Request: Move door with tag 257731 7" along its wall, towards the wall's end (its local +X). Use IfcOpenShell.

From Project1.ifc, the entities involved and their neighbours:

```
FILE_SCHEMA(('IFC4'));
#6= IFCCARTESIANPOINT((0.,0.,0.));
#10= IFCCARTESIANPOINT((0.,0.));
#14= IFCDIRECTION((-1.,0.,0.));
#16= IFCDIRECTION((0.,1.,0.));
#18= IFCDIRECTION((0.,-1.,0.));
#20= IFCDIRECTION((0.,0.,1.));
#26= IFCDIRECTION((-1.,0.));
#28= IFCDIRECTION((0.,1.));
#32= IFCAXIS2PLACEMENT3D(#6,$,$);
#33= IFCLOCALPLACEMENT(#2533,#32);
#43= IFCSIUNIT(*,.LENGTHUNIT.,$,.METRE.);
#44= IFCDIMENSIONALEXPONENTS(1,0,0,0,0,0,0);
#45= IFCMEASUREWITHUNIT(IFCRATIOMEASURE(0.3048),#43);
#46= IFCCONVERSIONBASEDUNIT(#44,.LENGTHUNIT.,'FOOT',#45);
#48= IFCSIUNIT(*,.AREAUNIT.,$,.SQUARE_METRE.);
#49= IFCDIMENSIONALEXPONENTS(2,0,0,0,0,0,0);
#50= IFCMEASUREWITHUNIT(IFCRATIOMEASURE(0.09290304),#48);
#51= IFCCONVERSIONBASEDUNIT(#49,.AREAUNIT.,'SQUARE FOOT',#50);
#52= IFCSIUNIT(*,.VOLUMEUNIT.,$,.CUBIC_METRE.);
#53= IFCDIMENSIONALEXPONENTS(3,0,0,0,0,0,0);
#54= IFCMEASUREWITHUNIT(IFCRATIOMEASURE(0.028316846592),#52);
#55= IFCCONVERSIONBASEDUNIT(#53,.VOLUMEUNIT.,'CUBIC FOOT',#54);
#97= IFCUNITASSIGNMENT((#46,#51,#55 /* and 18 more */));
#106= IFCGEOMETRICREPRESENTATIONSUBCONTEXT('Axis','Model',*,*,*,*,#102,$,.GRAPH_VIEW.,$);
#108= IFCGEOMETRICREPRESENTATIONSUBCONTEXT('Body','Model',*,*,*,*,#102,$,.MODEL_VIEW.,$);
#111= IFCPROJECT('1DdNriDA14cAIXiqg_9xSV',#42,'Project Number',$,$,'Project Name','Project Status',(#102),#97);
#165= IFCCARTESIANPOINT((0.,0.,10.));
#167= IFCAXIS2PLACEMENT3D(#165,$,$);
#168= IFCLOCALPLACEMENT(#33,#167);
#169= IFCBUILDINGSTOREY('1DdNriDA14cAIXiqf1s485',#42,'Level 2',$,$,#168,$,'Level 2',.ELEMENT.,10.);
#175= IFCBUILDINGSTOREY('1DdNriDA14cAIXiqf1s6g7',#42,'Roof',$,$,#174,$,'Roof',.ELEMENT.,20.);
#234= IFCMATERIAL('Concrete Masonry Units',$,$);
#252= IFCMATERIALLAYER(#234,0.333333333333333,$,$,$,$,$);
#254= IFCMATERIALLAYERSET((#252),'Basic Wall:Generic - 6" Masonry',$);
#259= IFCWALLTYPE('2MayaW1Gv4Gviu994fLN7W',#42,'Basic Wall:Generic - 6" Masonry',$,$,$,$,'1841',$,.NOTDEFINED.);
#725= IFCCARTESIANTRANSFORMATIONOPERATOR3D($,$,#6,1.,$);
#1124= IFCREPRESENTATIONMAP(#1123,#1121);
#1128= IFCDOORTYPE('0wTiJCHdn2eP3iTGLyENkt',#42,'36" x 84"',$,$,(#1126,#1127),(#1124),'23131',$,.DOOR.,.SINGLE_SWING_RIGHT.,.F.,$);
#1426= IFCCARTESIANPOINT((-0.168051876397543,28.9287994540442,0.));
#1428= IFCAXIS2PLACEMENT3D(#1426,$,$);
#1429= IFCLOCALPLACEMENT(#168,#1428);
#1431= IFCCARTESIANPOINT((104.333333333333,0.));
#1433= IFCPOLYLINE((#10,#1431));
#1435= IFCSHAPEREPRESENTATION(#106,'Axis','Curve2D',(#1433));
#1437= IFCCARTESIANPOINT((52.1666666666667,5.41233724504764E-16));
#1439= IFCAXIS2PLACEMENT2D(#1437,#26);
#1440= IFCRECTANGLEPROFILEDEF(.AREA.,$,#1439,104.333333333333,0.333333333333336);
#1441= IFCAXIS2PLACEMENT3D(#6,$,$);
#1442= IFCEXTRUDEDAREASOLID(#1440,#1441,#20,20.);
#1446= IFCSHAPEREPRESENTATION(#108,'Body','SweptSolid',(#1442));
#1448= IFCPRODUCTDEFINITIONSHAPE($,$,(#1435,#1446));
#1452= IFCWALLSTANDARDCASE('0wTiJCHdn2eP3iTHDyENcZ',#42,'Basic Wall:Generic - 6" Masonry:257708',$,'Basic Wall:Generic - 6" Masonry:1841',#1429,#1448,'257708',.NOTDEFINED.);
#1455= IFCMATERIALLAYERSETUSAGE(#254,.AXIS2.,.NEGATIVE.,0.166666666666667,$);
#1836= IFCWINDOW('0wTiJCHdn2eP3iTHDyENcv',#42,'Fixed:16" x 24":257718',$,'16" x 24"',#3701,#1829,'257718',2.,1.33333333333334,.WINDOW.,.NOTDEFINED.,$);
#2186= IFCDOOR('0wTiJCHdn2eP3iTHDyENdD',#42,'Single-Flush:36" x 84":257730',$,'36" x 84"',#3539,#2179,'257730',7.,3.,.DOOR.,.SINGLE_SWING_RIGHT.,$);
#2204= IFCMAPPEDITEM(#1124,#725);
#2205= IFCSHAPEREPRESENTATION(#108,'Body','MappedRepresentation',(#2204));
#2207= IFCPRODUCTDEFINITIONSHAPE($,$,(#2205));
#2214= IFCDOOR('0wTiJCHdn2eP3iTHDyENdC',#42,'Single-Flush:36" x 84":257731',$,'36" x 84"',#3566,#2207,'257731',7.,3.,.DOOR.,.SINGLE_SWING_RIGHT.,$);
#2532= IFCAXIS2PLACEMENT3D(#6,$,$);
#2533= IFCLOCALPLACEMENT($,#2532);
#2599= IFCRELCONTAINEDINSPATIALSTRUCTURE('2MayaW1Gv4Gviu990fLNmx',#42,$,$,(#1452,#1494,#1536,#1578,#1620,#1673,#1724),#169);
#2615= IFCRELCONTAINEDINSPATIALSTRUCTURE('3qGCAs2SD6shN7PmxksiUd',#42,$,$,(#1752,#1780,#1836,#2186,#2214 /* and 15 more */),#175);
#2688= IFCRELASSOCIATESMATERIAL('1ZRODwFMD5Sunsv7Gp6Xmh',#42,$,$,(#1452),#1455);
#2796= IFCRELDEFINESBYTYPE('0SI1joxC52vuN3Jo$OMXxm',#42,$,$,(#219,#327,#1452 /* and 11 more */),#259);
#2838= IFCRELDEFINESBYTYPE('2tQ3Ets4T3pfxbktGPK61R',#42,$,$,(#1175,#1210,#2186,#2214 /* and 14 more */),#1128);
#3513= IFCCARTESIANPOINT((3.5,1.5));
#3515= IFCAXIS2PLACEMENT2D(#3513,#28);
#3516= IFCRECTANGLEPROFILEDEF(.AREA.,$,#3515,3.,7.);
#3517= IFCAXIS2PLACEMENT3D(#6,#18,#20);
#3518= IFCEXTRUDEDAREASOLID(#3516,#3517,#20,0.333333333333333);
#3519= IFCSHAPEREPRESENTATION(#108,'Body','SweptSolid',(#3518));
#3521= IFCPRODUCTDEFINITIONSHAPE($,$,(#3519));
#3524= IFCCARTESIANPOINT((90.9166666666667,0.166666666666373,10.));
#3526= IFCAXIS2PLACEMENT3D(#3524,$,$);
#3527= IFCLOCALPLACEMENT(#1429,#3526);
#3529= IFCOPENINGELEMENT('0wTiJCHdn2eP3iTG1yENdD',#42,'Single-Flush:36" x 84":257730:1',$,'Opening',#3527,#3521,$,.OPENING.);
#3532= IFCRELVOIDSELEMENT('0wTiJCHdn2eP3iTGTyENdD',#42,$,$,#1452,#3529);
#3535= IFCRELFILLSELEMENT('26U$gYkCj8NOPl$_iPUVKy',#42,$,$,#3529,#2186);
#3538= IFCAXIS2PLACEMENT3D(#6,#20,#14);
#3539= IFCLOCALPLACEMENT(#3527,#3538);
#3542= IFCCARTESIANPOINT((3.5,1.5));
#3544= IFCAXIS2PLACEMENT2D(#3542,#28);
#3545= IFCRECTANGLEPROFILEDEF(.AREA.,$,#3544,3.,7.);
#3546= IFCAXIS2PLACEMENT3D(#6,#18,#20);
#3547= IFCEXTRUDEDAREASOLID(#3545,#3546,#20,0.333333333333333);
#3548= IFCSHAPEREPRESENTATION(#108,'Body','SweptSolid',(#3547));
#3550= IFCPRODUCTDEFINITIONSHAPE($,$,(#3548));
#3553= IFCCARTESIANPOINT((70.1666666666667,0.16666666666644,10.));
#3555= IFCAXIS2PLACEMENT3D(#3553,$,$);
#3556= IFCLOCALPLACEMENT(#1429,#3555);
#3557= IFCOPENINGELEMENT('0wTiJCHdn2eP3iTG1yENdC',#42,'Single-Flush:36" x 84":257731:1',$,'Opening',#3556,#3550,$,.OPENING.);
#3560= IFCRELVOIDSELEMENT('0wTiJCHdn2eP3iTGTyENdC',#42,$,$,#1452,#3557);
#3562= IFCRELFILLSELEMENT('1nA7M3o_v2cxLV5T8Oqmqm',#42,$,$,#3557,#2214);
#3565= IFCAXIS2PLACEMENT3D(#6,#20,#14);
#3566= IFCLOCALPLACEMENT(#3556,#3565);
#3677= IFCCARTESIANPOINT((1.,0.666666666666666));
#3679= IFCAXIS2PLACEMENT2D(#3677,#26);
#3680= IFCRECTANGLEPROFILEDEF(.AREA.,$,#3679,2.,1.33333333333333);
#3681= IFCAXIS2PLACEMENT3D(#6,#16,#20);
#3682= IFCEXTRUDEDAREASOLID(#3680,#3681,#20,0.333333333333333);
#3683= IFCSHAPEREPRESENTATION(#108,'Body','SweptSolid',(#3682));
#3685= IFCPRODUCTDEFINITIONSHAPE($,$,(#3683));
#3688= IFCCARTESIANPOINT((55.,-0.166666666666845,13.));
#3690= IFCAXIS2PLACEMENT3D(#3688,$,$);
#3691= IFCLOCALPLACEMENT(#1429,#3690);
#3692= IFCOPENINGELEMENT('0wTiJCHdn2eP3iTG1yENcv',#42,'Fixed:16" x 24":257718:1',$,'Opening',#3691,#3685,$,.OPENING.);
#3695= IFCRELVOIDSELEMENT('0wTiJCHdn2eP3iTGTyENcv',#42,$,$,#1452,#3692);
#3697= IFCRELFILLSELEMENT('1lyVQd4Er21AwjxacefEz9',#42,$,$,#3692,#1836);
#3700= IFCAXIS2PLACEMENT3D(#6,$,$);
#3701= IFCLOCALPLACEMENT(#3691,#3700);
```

```python
import ifcopenshell
import ifcopenshell.api.geometry
import ifcopenshell.util.placement
import ifcopenshell.util.unit

model = ifcopenshell.open("Project1.ifc")
unit_scale = ifcopenshell.util.unit.calculate_unit_scale(model)

door = model.by_guid("0wTiJCHdn2eP3iTHDyENdC")
opening = door.FillsVoids[0].RelatingOpeningElement
wall = opening.VoidsElements[0].RelatingBuildingElement

wall_matrix = ifcopenshell.util.placement.get_local_placement(wall.ObjectPlacement)
shift = wall_matrix[:3, 0] * 7 * 0.0254 / unit_scale
before = ifcopenshell.util.placement.get_local_placement(door.ObjectPlacement)[:3, 3].copy()

# The door is placed relative to its opening, so it follows when the opening moves.
matrix = ifcopenshell.util.placement.get_local_placement(opening.ObjectPlacement)
matrix[:3, 3] += shift
ifcopenshell.api.geometry.edit_object_placement(
    model, product=opening, matrix=matrix, is_si=False, should_transform_children=True
)

after = ifcopenshell.util.placement.get_local_placement(door.ObjectPlacement)[:3, 3]
print("door moved by", (after - before).round(3) + 0.0)

model.write("Project1_v2.ifc")
```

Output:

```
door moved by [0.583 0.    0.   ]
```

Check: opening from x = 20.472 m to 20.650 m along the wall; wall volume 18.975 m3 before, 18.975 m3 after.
